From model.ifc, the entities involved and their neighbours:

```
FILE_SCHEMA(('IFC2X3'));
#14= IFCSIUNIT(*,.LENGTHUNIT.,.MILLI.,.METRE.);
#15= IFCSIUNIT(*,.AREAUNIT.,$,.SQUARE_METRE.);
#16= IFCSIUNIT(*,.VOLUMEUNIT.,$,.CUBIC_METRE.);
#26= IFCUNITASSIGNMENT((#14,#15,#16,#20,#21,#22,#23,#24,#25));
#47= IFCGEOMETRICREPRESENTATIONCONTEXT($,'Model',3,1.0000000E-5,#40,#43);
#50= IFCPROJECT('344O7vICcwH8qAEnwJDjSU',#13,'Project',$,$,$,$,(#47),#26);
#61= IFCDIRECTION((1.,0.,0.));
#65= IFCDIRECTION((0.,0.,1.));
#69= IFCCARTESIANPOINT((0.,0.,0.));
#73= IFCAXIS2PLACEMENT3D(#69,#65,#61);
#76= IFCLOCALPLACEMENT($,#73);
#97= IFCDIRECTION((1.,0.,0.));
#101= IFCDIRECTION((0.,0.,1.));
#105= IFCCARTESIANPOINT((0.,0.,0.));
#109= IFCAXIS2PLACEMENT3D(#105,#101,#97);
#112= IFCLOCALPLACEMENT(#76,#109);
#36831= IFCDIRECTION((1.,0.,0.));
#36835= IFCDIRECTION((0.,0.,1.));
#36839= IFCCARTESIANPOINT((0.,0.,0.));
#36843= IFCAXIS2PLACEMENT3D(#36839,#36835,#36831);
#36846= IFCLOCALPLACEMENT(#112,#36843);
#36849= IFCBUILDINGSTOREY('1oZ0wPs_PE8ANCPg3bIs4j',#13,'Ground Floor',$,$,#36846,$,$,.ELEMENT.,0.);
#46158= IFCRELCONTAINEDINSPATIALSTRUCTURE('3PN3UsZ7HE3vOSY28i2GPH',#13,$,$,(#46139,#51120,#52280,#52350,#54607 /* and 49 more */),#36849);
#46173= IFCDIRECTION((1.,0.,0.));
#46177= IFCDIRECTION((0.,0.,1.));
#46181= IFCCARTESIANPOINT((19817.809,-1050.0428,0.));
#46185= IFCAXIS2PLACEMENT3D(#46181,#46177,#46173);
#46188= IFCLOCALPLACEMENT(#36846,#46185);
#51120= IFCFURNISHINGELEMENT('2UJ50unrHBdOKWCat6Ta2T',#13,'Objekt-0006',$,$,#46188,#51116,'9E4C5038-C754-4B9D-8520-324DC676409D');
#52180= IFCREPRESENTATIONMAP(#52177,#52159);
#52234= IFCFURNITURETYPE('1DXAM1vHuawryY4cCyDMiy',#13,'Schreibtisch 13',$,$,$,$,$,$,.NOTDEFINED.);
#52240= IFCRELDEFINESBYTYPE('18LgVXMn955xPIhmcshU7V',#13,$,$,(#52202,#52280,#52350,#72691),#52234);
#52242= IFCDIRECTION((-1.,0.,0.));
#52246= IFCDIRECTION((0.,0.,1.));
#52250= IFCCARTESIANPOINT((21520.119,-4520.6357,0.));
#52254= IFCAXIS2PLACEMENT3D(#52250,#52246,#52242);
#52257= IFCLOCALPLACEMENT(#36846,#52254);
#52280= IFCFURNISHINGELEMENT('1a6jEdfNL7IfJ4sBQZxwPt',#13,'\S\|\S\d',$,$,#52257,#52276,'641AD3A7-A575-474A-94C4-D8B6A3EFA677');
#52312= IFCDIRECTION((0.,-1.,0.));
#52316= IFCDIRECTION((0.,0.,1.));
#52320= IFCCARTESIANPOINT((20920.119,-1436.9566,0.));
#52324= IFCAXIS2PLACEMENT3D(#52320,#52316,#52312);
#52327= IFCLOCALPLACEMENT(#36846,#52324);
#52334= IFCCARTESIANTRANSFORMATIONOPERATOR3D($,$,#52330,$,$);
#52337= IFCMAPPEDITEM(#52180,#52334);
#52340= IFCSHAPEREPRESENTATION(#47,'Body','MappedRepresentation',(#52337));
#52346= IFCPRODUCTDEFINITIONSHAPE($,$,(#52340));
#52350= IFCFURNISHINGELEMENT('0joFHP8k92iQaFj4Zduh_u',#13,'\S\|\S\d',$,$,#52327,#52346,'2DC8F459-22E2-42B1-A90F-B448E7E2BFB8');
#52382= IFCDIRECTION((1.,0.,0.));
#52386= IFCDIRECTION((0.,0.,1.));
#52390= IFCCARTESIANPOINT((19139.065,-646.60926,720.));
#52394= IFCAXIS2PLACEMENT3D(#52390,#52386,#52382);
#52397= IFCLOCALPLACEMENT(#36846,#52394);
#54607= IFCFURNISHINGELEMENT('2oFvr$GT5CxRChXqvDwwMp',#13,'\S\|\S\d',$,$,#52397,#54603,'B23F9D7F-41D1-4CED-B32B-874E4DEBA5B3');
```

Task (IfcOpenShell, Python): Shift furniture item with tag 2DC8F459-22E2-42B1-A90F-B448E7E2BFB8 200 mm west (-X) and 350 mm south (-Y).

```python
import ifcopenshell
import ifcopenshell.api.geometry
import ifcopenshell.util.placement
import ifcopenshell.util.unit

model = ifcopenshell.open("model.ifc")
unit_scale = ifcopenshell.util.unit.calculate_unit_scale(model)

item = model.by_guid("0joFHP8k92iQaFj4Zduh_u")
matrix = ifcopenshell.util.placement.get_local_placement(item.ObjectPlacement)
matrix[0, 3] -= 0.2 / unit_scale
matrix[1, 3] -= 0.35 / unit_scale
ifcopenshell.api.geometry.edit_object_placement(model, product=item, matrix=matrix, is_si=False)

print(ifcopenshell.util.placement.get_local_placement(item.ObjectPlacement).round(3) + 0.0)

model.write("model-out.ifc")
```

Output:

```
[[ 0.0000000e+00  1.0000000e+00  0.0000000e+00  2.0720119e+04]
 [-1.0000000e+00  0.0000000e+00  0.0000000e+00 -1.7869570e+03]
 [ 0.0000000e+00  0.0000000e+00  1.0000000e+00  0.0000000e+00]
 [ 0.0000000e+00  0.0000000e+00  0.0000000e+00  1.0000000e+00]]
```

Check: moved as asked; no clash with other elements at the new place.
